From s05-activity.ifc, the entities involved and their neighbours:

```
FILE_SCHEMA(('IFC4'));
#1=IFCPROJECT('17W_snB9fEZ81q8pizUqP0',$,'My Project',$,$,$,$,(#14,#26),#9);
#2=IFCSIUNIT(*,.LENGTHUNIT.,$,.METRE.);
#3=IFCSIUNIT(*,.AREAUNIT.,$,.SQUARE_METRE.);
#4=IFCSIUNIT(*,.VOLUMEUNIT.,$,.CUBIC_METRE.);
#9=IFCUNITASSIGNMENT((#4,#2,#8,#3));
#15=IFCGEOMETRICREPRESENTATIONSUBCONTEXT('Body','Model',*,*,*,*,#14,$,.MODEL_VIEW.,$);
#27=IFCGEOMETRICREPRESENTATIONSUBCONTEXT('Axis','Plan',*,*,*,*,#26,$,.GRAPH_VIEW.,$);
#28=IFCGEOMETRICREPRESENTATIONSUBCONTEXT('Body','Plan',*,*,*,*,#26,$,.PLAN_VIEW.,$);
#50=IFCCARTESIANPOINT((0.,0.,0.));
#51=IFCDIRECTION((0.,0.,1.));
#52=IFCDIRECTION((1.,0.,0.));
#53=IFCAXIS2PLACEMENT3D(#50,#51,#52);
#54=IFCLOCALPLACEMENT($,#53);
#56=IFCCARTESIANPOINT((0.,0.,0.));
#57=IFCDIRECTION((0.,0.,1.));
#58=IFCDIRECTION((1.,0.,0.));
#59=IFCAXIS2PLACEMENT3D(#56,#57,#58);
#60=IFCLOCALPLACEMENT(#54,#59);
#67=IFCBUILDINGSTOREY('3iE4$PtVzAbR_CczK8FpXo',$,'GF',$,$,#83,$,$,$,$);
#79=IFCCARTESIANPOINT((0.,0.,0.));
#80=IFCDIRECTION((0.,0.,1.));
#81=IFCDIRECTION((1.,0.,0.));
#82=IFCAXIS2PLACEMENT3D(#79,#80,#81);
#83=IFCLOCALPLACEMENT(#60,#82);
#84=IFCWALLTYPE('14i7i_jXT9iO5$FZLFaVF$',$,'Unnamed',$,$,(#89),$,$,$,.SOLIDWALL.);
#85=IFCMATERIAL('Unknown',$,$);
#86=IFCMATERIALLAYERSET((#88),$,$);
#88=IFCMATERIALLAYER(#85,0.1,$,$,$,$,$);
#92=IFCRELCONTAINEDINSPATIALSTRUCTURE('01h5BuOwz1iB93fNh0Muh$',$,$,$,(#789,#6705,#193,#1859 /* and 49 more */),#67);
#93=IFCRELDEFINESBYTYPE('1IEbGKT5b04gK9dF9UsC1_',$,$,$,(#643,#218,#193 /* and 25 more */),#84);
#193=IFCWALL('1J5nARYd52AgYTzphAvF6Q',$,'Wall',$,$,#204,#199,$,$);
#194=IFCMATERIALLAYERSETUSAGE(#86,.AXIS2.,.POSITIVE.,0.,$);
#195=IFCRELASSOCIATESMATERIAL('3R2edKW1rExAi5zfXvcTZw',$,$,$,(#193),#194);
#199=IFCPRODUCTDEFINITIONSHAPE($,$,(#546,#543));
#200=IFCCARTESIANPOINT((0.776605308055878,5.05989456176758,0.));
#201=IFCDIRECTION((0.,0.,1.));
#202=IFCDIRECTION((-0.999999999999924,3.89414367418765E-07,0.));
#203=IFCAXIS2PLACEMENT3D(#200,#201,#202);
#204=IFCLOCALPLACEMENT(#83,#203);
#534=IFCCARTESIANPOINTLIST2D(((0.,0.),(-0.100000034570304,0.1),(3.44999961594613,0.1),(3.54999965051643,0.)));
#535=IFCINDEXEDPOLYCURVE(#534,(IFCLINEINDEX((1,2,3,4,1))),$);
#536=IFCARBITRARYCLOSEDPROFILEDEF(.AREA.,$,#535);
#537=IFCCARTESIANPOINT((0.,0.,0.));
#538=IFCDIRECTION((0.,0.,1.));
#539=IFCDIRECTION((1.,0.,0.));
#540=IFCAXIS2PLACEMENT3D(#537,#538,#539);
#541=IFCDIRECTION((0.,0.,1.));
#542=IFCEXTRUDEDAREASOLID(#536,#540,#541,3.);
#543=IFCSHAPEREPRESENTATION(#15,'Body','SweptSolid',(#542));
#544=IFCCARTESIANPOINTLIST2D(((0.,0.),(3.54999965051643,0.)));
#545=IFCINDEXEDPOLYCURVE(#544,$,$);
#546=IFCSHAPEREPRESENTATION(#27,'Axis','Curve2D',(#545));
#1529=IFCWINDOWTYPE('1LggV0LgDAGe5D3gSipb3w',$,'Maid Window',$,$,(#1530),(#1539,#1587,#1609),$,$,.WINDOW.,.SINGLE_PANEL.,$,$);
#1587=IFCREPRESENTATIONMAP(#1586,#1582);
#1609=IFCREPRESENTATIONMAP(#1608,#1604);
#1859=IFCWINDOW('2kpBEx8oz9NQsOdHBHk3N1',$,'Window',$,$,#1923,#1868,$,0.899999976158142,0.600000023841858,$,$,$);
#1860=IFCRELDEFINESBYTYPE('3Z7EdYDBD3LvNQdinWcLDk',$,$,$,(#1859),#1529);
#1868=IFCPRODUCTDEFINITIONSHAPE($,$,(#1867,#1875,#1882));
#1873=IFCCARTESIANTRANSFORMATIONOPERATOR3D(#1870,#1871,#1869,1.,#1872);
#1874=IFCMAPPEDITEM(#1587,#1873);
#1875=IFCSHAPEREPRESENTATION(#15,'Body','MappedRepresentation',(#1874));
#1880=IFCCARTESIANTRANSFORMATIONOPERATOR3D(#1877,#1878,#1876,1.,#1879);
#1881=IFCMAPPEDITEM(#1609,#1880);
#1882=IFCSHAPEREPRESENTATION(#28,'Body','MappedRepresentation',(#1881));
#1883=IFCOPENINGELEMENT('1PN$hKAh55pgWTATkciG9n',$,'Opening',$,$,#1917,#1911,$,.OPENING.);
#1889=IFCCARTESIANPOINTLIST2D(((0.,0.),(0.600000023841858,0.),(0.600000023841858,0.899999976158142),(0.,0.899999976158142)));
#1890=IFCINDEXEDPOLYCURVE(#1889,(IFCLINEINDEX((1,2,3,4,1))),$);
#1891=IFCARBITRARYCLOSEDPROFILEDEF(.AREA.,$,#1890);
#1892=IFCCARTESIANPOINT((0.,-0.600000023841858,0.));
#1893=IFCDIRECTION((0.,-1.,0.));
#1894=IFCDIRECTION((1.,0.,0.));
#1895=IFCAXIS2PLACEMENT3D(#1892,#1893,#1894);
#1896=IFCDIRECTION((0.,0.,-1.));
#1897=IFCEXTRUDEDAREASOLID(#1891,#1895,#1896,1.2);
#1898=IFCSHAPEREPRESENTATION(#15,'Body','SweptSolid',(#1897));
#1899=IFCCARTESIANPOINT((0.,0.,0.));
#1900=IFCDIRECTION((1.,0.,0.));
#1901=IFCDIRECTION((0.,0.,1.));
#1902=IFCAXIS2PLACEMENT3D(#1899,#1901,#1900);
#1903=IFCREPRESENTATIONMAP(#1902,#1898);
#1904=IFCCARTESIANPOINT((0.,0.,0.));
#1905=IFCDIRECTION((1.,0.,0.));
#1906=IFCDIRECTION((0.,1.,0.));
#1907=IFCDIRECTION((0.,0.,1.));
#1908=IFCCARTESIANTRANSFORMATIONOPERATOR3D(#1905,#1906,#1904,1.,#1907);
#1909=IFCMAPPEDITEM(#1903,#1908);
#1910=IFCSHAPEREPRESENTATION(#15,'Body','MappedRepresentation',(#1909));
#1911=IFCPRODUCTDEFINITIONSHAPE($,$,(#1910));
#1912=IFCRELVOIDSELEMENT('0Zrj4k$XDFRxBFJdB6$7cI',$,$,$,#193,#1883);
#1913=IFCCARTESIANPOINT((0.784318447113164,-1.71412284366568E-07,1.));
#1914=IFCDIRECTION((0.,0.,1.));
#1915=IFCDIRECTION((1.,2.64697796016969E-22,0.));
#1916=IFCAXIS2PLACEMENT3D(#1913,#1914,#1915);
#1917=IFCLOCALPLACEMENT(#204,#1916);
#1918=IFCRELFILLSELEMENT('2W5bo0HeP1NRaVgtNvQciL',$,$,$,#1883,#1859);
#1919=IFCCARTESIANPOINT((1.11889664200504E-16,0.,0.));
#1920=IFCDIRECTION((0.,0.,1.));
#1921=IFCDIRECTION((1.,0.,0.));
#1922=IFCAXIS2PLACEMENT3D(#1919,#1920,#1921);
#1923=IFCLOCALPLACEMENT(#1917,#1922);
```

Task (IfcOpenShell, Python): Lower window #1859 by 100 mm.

```python
import numpy as np
import ifcopenshell
import ifcopenshell.api.geometry
import ifcopenshell.util.placement
import ifcopenshell.util.unit

model = ifcopenshell.open("s05-activity.ifc")
unit_scale = ifcopenshell.util.unit.calculate_unit_scale(model)

window = model.by_id(1859)
opening = window.FillsVoids[0].RelatingOpeningElement
dz = -0.1 / unit_scale

shift = np.array([0.0, 0.0, dz])
# The window is placed relative to its opening, so it follows when the opening moves.
matrix = ifcopenshell.util.placement.get_local_placement(opening.ObjectPlacement)
matrix[:3, 3] += shift
ifcopenshell.api.geometry.edit_object_placement(
    model, product=opening, matrix=matrix, is_si=False, should_transform_children=True
)

print(f"moved by {dz * unit_scale:+.3f} m")

model.write("s05-activity-out.ifc")
```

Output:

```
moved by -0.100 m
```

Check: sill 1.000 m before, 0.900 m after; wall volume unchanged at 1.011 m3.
